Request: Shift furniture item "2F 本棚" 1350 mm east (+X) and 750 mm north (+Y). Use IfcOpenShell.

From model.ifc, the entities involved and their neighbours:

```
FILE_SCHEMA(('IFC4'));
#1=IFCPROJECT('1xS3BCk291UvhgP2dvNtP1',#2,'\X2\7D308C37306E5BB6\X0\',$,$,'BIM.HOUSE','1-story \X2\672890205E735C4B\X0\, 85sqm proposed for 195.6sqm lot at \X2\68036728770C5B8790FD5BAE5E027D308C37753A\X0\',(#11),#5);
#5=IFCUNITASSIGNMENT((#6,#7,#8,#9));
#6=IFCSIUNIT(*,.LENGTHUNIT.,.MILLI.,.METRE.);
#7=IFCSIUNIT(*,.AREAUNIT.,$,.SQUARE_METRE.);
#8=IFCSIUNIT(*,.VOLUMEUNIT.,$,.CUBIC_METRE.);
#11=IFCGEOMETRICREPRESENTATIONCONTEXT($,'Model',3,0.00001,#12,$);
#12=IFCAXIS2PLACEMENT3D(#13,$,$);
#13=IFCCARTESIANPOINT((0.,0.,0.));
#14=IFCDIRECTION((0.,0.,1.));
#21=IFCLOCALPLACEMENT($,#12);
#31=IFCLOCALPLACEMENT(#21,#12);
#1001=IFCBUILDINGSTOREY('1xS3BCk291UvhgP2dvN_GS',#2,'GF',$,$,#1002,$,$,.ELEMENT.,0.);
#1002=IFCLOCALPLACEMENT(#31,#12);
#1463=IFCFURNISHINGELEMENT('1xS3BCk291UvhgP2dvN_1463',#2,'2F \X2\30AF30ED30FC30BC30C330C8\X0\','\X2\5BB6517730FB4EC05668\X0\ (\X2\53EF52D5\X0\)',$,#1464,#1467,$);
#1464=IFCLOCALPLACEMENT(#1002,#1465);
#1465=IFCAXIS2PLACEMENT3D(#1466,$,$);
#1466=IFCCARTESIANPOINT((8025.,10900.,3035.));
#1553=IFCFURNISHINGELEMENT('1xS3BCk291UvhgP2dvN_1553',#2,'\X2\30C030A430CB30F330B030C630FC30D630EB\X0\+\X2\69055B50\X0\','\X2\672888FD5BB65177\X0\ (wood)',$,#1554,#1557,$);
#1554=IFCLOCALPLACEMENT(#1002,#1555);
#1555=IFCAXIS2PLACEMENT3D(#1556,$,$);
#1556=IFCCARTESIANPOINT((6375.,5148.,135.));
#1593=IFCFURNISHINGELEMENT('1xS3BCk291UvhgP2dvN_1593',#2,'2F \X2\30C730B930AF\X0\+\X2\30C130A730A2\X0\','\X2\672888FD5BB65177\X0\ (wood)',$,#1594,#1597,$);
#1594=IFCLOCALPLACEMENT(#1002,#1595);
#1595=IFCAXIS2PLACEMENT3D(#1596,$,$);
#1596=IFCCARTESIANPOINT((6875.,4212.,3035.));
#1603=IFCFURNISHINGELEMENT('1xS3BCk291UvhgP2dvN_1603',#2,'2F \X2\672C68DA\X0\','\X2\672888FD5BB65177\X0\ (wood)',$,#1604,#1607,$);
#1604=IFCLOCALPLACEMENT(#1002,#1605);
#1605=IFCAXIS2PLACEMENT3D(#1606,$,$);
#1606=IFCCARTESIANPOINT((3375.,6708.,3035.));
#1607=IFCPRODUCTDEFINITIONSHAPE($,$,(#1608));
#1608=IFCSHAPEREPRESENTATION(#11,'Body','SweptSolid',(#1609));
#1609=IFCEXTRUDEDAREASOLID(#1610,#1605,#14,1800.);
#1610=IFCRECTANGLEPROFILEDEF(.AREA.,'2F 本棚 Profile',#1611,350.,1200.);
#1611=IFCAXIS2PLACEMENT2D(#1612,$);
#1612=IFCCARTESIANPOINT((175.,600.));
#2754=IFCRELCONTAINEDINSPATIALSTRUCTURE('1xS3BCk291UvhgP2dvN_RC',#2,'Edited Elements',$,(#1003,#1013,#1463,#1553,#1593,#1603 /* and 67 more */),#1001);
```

```python
import ifcopenshell
import ifcopenshell.api.geometry
import ifcopenshell.util.placement
import ifcopenshell.util.unit

model = ifcopenshell.open("model.ifc")
unit_scale = ifcopenshell.util.unit.calculate_unit_scale(model)

item = model.by_id(1603)
matrix = ifcopenshell.util.placement.get_local_placement(item.ObjectPlacement)
matrix[0, 3] += 1.35 / unit_scale
matrix[1, 3] += 0.75 / unit_scale
ifcopenshell.api.geometry.edit_object_placement(model, product=item, matrix=matrix, is_si=False)

print(ifcopenshell.util.placement.get_local_placement(item.ObjectPlacement).round(3) + 0.0)

model.write("model_rev.ifc")
```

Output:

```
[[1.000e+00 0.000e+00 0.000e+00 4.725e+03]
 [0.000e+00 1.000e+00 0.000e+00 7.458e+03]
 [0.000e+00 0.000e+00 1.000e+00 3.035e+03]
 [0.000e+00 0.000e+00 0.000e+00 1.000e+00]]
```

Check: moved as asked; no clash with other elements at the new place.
